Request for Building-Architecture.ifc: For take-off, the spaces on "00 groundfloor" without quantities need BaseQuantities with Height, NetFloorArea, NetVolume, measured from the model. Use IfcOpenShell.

First a look at what the model holds.

```python
import ifcopenshell
import ifcopenshell.util.element
import ifcopenshell.util.unit

model = ifcopenshell.open("Building-Architecture.ifc")
print(model.schema)
for unit_type in ("LENGTHUNIT", "AREAUNIT", "VOLUMEUNIT"):
    print(unit_type, ifcopenshell.util.unit.calculate_unit_scale(model, unit_type))
storey = next(s for s in model.by_type("IfcBuildingStorey") if s.Name == "00 groundfloor")
spaces = [e for e in ifcopenshell.util.element.get_decomposition(storey) if e.is_a("IfcSpace")]
for e in sorted(spaces, key=lambda e: e.id()):
    print(e.id(), e.is_a(), e.Name, list(ifcopenshell.util.element.get_psets(e, qtos_only=True)), sep=" | ")
```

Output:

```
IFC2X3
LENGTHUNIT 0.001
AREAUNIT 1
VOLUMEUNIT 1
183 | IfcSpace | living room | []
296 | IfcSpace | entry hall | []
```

```python
import ifcopenshell
import ifcopenshell.api.pset
import ifcopenshell.geom
import ifcopenshell.util.element
import ifcopenshell.util.shape
import ifcopenshell.util.unit

model = ifcopenshell.open("Building-Architecture.ifc")
unit_scale = ifcopenshell.util.unit.calculate_unit_scale(model)
area_scale = ifcopenshell.util.unit.calculate_unit_scale(model, "AREAUNIT")
volume_scale = ifcopenshell.util.unit.calculate_unit_scale(model, "VOLUMEUNIT")
settings = ifcopenshell.geom.settings()

storey = next(s for s in model.by_type("IfcBuildingStorey") if s.Name == "00 groundfloor")
spaces = [e for e in ifcopenshell.util.element.get_decomposition(storey) if e.is_a("IfcSpace")]

for e in sorted(spaces, key=lambda e: e.id()):
    if ifcopenshell.util.element.get_psets(e, qtos_only=True, should_inherit=False):
        continue
    # Geometry comes back in metres, in the element's own axes.
    shape = ifcopenshell.geom.create_shape(settings, e)
    values = {
        "Height": ifcopenshell.util.shape.get_z(shape.geometry) / unit_scale,
        "NetFloorArea": ifcopenshell.util.shape.get_footprint_area(shape.geometry) / area_scale,
        "NetVolume": ifcopenshell.util.shape.get_volume(shape.geometry) / volume_scale,
    }
    qto = ifcopenshell.api.pset.add_qto(model, product=e, name="BaseQuantities")
    ifcopenshell.api.pset.edit_qto(model, qto=qto, properties=values)
    print(e.id(), {k: round(v, 3) for k, v in values.items()})

model.write("Building-Architecture_rev.ifc")
```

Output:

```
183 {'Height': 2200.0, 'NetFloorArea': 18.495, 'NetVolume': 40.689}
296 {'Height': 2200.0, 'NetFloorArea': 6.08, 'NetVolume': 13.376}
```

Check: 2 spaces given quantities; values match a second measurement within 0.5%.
